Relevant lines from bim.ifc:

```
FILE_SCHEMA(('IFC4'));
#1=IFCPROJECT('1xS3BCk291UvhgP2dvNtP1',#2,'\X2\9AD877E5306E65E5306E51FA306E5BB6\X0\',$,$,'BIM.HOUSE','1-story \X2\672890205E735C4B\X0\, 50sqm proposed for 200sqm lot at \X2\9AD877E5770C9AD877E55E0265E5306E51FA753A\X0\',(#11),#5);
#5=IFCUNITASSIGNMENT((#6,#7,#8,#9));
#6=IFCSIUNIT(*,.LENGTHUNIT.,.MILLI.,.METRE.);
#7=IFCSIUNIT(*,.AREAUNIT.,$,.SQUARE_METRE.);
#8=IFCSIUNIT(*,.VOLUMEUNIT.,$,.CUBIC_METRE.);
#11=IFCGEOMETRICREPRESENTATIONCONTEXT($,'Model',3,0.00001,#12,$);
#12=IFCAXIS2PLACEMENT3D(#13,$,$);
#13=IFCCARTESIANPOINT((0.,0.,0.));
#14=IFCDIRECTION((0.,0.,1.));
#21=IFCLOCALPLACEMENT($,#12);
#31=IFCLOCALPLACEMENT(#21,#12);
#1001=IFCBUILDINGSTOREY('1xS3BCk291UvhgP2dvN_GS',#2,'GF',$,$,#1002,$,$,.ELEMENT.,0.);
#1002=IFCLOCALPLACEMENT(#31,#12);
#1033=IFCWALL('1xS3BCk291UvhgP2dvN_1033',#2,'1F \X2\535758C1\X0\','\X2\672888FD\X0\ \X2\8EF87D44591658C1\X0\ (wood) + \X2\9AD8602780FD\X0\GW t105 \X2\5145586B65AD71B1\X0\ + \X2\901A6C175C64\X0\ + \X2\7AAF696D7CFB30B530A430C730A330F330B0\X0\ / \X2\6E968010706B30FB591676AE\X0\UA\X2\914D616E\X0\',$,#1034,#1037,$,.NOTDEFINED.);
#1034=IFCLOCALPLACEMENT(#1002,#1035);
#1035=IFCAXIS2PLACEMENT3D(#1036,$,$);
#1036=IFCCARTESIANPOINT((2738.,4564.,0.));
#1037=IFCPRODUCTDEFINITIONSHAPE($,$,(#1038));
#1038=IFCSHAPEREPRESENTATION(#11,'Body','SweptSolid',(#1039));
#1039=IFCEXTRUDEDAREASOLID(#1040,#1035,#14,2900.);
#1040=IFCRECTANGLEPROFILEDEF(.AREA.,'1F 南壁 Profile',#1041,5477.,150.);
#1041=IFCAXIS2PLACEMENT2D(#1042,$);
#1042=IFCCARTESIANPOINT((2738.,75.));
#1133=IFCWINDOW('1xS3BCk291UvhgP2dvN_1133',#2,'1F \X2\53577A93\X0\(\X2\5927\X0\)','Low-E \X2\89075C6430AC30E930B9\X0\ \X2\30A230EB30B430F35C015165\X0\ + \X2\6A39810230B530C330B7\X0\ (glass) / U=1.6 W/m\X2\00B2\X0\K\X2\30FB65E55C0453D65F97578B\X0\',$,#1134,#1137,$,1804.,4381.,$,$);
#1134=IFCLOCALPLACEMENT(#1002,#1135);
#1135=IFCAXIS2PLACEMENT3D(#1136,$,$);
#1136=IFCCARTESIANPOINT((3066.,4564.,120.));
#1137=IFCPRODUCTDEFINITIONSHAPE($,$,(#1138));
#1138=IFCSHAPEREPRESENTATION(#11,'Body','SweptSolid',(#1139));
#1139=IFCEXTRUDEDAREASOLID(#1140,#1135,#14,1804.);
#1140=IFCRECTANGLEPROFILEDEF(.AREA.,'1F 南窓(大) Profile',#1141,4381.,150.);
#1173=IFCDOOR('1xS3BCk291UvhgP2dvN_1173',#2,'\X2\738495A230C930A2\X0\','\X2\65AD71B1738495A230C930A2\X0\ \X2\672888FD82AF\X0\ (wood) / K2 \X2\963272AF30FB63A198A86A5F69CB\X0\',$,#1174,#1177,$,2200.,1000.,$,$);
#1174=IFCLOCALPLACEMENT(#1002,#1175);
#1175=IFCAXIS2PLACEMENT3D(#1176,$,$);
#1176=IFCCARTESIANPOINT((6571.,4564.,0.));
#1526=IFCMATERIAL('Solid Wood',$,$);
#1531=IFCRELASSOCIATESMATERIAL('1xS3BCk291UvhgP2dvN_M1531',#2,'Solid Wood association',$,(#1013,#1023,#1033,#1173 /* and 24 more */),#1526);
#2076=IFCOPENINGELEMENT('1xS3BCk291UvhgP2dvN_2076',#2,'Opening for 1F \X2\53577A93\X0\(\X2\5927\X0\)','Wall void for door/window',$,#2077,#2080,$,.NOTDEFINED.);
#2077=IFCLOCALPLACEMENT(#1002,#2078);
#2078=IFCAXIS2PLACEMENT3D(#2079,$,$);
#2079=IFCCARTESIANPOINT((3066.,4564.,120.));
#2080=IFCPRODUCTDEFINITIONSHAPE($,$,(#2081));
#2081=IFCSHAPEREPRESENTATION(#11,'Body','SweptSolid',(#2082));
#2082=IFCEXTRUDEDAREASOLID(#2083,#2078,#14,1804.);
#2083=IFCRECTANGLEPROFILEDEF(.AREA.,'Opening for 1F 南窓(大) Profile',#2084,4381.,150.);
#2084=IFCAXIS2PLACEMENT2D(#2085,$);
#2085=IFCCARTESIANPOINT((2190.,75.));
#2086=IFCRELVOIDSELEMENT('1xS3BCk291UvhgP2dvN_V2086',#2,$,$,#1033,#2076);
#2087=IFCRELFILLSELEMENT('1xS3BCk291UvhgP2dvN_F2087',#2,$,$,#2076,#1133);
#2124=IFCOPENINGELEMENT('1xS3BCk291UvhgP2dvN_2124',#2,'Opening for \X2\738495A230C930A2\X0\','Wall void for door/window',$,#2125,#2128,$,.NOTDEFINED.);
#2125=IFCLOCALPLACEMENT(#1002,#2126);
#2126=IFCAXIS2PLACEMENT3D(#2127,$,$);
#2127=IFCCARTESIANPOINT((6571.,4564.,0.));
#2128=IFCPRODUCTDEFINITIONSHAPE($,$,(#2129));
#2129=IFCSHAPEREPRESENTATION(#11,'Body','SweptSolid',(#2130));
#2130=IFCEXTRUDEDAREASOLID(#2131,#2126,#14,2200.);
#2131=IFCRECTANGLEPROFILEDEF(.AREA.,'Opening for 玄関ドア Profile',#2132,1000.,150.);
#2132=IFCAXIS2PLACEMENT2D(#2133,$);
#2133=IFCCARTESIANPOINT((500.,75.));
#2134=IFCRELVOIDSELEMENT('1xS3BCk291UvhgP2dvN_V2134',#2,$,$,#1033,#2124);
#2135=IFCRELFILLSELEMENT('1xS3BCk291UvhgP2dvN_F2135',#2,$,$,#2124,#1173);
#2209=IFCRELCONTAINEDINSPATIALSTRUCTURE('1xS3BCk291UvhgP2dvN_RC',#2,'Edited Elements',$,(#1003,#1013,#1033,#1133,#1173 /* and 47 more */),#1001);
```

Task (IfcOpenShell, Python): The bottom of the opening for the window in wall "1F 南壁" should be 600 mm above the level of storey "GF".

```python
import numpy as np
import ifcopenshell
import ifcopenshell.api.geometry
import ifcopenshell.geom
import ifcopenshell.util.element
import ifcopenshell.util.placement
import ifcopenshell.util.shape
import ifcopenshell.util.unit

model = ifcopenshell.open("bim.ifc")
unit_scale = ifcopenshell.util.unit.calculate_unit_scale(model)

window = model.by_guid("1xS3BCk291UvhgP2dvN_1133")
opening = window.FillsVoids[0].RelatingOpeningElement
storey = ifcopenshell.util.element.get_container(window, ifc_class="IfcBuildingStorey")
level = ifcopenshell.util.placement.get_local_placement(storey.ObjectPlacement)[2, 3]

# The opening's origin need not be at the sill, so measure its lowest point.
shape = ifcopenshell.geom.create_shape(ifcopenshell.geom.settings(), opening)
bottom = ifcopenshell.util.shape.get_shape_bottom_elevation(shape, shape.geometry) / unit_scale
dz = level + 0.6 / unit_scale - bottom

shift = np.array([0.0, 0.0, dz])
# The window is not placed relative to its opening, so move both.
for product in (opening, window):
    matrix = ifcopenshell.util.placement.get_local_placement(product.ObjectPlacement)
    matrix[:3, 3] += shift
    ifcopenshell.api.geometry.edit_object_placement(model, product=product, matrix=matrix, is_si=False)

print(f"moved by {dz * unit_scale:+.3f} m")

model.write("bim_v2.ifc")
```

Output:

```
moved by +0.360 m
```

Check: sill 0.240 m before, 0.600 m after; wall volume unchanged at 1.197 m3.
